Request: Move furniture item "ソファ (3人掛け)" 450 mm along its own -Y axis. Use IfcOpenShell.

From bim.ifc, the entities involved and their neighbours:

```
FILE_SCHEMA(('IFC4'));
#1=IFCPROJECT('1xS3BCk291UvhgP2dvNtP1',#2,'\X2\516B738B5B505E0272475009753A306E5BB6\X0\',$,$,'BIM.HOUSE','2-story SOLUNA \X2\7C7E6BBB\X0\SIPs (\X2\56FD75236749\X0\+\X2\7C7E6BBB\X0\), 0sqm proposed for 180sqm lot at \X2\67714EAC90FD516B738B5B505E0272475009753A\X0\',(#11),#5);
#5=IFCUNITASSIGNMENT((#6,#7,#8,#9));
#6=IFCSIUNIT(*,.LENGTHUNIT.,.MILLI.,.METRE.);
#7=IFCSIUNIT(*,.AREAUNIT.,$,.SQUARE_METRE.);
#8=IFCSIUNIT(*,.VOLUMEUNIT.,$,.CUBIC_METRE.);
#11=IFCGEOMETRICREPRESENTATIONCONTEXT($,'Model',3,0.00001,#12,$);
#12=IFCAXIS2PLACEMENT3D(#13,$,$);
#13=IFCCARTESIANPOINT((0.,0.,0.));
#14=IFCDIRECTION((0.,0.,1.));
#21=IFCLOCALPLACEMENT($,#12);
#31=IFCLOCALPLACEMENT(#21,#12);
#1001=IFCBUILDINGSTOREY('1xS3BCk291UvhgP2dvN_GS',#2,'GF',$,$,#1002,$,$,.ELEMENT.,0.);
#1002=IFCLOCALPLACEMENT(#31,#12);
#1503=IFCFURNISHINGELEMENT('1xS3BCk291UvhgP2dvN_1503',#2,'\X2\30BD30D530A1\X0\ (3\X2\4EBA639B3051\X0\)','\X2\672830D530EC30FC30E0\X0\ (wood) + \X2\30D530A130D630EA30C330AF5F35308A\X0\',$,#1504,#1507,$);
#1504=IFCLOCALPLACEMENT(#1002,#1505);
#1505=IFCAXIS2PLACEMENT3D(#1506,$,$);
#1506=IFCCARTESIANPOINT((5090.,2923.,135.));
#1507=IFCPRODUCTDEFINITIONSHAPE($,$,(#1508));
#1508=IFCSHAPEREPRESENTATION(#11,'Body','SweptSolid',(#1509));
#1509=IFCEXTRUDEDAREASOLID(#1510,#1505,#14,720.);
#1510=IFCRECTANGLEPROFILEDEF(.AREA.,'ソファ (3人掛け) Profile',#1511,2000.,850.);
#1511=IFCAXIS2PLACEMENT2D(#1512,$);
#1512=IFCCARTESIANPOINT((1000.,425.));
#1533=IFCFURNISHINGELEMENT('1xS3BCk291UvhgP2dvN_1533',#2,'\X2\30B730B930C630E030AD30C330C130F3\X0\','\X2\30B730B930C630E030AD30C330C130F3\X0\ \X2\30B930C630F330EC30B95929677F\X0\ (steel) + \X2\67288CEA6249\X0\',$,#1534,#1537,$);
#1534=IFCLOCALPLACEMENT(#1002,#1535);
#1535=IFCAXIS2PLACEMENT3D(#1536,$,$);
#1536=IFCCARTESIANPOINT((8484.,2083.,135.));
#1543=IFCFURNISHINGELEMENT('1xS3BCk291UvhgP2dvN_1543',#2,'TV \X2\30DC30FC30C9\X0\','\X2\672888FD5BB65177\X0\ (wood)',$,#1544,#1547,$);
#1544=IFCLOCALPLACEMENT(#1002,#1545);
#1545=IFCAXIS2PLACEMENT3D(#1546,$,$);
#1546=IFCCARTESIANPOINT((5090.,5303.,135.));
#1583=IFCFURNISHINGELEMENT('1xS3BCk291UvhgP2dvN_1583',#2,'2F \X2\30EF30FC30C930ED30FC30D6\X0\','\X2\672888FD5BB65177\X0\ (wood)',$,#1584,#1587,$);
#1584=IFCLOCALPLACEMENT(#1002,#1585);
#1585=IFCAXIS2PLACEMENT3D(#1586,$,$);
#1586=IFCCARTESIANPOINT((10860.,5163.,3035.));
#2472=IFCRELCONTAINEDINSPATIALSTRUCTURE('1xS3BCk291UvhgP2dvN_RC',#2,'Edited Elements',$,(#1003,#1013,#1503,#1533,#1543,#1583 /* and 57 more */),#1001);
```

```python
import ifcopenshell
import ifcopenshell.api.geometry
import ifcopenshell.util.placement

model = ifcopenshell.open("bim.ifc")

item = model.by_id(1503)
matrix = ifcopenshell.util.placement.get_local_placement(item.ObjectPlacement)
matrix[:3, 3] -= matrix[:3, 1] * 450.0
ifcopenshell.api.geometry.edit_object_placement(model, product=item, matrix=matrix, is_si=False)

print(ifcopenshell.util.placement.get_local_placement(item.ObjectPlacement).round(3) + 0.0)

model.write("bim_rev.ifc")
```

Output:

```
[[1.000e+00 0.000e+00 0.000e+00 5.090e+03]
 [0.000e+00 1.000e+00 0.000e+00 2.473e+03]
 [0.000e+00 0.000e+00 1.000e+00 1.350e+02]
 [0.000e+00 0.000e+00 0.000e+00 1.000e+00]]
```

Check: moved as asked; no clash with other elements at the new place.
